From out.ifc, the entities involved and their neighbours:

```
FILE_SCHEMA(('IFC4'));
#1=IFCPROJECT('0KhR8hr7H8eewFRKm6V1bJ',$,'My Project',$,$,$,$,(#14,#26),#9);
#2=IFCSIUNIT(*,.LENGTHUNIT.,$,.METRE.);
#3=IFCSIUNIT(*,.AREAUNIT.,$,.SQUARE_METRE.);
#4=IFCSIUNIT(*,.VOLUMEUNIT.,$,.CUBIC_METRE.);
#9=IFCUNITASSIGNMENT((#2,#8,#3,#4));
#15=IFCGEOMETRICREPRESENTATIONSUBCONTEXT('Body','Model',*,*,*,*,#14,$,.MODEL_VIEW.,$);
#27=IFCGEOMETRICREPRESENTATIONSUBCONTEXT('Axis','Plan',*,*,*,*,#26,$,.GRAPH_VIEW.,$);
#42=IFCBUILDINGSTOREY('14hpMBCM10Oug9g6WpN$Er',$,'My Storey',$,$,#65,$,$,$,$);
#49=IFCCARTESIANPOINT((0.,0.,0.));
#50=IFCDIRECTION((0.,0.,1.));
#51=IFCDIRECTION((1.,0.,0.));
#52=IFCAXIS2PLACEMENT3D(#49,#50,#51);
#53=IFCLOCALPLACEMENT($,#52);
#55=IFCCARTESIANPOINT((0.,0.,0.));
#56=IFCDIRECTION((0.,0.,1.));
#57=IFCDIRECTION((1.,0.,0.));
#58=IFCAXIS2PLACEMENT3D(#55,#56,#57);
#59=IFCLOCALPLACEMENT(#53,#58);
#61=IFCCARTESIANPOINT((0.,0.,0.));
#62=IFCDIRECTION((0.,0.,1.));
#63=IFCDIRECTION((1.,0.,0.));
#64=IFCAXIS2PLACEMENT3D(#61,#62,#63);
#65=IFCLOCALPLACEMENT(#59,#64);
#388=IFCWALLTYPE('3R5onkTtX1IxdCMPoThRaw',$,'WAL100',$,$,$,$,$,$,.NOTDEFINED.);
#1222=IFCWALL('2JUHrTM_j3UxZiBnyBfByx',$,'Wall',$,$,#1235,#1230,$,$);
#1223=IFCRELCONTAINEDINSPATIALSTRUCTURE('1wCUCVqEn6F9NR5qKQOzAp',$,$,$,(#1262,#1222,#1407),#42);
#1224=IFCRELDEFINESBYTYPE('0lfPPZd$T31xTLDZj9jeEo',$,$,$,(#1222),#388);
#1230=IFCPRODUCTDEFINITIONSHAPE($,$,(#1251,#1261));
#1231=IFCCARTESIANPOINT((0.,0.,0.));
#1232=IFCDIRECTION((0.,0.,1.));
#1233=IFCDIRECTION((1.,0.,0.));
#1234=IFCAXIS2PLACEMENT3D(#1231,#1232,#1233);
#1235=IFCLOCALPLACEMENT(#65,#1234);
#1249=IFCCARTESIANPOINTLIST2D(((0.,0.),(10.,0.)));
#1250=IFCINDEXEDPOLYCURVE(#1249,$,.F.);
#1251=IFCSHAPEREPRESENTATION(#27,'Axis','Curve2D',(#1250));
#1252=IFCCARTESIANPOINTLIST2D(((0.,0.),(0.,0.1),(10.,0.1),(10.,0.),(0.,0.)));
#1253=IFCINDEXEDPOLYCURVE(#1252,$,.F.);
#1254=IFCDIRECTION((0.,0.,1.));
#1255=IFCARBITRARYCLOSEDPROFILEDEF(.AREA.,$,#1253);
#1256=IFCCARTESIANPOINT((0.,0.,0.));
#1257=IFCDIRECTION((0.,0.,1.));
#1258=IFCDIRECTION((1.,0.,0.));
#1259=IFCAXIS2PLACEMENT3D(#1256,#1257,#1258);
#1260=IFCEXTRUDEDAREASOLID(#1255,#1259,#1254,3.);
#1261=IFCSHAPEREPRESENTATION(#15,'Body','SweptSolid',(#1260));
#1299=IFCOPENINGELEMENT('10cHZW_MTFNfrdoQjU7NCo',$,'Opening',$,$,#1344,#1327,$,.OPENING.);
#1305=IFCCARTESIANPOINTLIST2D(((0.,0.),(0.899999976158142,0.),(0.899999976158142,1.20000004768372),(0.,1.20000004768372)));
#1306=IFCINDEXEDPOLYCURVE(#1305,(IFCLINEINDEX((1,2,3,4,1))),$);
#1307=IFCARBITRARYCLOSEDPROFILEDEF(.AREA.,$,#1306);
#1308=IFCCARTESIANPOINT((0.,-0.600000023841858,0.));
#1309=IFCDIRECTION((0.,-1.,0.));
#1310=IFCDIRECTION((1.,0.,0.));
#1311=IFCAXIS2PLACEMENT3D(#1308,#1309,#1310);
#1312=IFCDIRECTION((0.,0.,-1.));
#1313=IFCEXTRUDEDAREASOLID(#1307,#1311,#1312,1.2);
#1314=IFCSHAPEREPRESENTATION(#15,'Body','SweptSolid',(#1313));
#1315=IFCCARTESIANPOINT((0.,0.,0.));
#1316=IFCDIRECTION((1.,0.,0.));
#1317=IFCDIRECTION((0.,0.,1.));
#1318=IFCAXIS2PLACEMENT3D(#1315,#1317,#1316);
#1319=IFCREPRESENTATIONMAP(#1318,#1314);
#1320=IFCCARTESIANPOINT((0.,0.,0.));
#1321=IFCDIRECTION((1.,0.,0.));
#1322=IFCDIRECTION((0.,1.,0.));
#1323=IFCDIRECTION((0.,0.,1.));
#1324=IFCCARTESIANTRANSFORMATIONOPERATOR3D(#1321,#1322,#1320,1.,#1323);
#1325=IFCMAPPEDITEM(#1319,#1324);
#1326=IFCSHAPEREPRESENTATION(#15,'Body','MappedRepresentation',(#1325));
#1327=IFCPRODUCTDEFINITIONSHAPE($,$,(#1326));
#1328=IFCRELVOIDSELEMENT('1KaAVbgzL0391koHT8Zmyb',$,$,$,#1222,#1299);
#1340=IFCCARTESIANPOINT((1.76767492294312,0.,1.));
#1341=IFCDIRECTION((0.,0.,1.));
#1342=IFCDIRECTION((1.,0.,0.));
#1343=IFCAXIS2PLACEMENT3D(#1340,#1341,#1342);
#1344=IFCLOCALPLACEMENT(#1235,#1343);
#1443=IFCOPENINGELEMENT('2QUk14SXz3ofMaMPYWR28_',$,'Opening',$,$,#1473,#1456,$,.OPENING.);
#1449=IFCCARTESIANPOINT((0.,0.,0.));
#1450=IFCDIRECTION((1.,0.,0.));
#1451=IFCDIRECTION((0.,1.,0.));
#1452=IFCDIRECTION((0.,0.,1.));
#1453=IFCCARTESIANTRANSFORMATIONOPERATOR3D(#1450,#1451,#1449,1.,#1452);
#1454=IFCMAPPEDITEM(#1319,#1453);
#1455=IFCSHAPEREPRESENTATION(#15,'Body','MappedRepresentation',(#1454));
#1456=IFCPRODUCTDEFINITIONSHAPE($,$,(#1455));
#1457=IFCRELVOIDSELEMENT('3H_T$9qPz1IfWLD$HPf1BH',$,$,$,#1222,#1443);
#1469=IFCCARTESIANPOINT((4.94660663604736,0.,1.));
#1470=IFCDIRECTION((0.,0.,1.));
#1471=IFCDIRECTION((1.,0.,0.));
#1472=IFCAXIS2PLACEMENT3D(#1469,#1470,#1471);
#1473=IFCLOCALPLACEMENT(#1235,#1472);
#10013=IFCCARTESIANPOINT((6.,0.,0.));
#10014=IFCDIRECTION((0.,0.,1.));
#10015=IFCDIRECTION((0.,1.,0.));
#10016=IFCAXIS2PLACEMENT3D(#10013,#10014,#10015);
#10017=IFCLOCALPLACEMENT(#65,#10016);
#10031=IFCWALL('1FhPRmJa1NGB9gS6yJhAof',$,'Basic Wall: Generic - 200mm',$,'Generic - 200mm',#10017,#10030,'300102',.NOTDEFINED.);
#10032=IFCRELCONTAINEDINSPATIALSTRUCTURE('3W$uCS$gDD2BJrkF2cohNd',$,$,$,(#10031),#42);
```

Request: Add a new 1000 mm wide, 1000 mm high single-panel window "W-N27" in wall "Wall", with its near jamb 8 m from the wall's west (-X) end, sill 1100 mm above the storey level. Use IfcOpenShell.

```python
import numpy as np
import ifcopenshell
import ifcopenshell.api.feature
import ifcopenshell.api.geometry
import ifcopenshell.api.root
import ifcopenshell.api.spatial
import ifcopenshell.geom
import ifcopenshell.util.element
import ifcopenshell.util.placement
import ifcopenshell.util.representation
import ifcopenshell.util.shape
import ifcopenshell.util.unit

model = ifcopenshell.open("out.ifc")
unit_scale = ifcopenshell.util.unit.calculate_unit_scale(model)
settings = ifcopenshell.geom.settings()


def volume(element):
    """Net volume in cubic metres, openings subtracted."""
    shape = ifcopenshell.geom.create_shape(settings, element)
    return ifcopenshell.util.shape.get_volume(shape.geometry)


wall = model.by_guid("2JUHrTM_j3UxZiBnyBfByx")
storey = ifcopenshell.util.element.get_container(wall, ifc_class="IfcBuildingStorey")
context = ifcopenshell.util.representation.get_context(model, "Model", "Body", "MODEL_VIEW")
before = volume(wall)

width, height, from_end, sill = 1, 1, 8, 1.1  # metres

# The wall runs along its own X axis, and the end named is its -X end.
wall_shape = ifcopenshell.geom.create_shape(settings, wall)
x, y, z = ifcopenshell.util.shape.get_vertices(wall_shape.geometry).T
start = x.min() + from_end
face, thickness = float(y.min()), float(y.max() - y.min())
wall_matrix = ifcopenshell.util.placement.get_local_placement(wall.ObjectPlacement)
level = ifcopenshell.util.placement.get_local_placement(storey.ObjectPlacement)[2, 3]


def in_wall(x, y):
    """Placement at x, y metres in the wall's axes, at sill height."""
    matrix = wall_matrix.copy()
    matrix[:, 3] = wall_matrix @ np.array([x / unit_scale, y / unit_scale, 0.0, 1.0])
    matrix[2, 3] = level + sill / unit_scale
    return matrix


# Opening: a box that overshoots both wall faces by 50 mm.
opening = ifcopenshell.api.root.create_entity(model, ifc_class="IfcOpeningElement", predefined_type="OPENING")
box = ifcopenshell.api.geometry.add_wall_representation(
    model, context=context, length=width, height=height, thickness=thickness + 0.1
)
ifcopenshell.api.geometry.assign_representation(model, product=opening, representation=box)
ifcopenshell.api.geometry.edit_object_placement(model, product=opening, matrix=in_wall(start, face - 0.05), is_si=False)
ifcopenshell.api.feature.add_feature(model, feature=opening, element=wall)

window = ifcopenshell.api.root.create_entity(model, ifc_class="IfcWindow", name="W-N27", predefined_type="WINDOW")
window.OverallWidth, window.OverallHeight = width / unit_scale, height / unit_scale
window.PartitioningType = "SINGLE_PANEL"
body = ifcopenshell.api.geometry.add_window_representation(
    model,
    context=context,
    overall_width=window.OverallWidth,
    overall_height=window.OverallHeight,
    partition_type="SINGLE_PANEL",
)
ifcopenshell.api.geometry.assign_representation(model, product=window, representation=body)
ifcopenshell.api.spatial.assign_container(model, products=[window], relating_structure=storey)
ifcopenshell.api.feature.add_filling(model, opening=opening, element=window)

# Centre the window in the wall's thickness.
ifcopenshell.api.geometry.edit_object_placement(model, product=window, matrix=in_wall(start, face), is_si=False)
window_shape = ifcopenshell.geom.create_shape(settings, window)
depth = ifcopenshell.util.shape.get_vertices(window_shape.geometry)[:, 1]
offset = face + thickness / 2 - (depth.min() + depth.max()) / 2
ifcopenshell.api.geometry.edit_object_placement(model, product=window, matrix=in_wall(start, offset), is_si=False)

after = volume(wall)

print(f"wall volume {before:.3f} -> {after:.3f} m3")

model.write("out_updated.ifc")
```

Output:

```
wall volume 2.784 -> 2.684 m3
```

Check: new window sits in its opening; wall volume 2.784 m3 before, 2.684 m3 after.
